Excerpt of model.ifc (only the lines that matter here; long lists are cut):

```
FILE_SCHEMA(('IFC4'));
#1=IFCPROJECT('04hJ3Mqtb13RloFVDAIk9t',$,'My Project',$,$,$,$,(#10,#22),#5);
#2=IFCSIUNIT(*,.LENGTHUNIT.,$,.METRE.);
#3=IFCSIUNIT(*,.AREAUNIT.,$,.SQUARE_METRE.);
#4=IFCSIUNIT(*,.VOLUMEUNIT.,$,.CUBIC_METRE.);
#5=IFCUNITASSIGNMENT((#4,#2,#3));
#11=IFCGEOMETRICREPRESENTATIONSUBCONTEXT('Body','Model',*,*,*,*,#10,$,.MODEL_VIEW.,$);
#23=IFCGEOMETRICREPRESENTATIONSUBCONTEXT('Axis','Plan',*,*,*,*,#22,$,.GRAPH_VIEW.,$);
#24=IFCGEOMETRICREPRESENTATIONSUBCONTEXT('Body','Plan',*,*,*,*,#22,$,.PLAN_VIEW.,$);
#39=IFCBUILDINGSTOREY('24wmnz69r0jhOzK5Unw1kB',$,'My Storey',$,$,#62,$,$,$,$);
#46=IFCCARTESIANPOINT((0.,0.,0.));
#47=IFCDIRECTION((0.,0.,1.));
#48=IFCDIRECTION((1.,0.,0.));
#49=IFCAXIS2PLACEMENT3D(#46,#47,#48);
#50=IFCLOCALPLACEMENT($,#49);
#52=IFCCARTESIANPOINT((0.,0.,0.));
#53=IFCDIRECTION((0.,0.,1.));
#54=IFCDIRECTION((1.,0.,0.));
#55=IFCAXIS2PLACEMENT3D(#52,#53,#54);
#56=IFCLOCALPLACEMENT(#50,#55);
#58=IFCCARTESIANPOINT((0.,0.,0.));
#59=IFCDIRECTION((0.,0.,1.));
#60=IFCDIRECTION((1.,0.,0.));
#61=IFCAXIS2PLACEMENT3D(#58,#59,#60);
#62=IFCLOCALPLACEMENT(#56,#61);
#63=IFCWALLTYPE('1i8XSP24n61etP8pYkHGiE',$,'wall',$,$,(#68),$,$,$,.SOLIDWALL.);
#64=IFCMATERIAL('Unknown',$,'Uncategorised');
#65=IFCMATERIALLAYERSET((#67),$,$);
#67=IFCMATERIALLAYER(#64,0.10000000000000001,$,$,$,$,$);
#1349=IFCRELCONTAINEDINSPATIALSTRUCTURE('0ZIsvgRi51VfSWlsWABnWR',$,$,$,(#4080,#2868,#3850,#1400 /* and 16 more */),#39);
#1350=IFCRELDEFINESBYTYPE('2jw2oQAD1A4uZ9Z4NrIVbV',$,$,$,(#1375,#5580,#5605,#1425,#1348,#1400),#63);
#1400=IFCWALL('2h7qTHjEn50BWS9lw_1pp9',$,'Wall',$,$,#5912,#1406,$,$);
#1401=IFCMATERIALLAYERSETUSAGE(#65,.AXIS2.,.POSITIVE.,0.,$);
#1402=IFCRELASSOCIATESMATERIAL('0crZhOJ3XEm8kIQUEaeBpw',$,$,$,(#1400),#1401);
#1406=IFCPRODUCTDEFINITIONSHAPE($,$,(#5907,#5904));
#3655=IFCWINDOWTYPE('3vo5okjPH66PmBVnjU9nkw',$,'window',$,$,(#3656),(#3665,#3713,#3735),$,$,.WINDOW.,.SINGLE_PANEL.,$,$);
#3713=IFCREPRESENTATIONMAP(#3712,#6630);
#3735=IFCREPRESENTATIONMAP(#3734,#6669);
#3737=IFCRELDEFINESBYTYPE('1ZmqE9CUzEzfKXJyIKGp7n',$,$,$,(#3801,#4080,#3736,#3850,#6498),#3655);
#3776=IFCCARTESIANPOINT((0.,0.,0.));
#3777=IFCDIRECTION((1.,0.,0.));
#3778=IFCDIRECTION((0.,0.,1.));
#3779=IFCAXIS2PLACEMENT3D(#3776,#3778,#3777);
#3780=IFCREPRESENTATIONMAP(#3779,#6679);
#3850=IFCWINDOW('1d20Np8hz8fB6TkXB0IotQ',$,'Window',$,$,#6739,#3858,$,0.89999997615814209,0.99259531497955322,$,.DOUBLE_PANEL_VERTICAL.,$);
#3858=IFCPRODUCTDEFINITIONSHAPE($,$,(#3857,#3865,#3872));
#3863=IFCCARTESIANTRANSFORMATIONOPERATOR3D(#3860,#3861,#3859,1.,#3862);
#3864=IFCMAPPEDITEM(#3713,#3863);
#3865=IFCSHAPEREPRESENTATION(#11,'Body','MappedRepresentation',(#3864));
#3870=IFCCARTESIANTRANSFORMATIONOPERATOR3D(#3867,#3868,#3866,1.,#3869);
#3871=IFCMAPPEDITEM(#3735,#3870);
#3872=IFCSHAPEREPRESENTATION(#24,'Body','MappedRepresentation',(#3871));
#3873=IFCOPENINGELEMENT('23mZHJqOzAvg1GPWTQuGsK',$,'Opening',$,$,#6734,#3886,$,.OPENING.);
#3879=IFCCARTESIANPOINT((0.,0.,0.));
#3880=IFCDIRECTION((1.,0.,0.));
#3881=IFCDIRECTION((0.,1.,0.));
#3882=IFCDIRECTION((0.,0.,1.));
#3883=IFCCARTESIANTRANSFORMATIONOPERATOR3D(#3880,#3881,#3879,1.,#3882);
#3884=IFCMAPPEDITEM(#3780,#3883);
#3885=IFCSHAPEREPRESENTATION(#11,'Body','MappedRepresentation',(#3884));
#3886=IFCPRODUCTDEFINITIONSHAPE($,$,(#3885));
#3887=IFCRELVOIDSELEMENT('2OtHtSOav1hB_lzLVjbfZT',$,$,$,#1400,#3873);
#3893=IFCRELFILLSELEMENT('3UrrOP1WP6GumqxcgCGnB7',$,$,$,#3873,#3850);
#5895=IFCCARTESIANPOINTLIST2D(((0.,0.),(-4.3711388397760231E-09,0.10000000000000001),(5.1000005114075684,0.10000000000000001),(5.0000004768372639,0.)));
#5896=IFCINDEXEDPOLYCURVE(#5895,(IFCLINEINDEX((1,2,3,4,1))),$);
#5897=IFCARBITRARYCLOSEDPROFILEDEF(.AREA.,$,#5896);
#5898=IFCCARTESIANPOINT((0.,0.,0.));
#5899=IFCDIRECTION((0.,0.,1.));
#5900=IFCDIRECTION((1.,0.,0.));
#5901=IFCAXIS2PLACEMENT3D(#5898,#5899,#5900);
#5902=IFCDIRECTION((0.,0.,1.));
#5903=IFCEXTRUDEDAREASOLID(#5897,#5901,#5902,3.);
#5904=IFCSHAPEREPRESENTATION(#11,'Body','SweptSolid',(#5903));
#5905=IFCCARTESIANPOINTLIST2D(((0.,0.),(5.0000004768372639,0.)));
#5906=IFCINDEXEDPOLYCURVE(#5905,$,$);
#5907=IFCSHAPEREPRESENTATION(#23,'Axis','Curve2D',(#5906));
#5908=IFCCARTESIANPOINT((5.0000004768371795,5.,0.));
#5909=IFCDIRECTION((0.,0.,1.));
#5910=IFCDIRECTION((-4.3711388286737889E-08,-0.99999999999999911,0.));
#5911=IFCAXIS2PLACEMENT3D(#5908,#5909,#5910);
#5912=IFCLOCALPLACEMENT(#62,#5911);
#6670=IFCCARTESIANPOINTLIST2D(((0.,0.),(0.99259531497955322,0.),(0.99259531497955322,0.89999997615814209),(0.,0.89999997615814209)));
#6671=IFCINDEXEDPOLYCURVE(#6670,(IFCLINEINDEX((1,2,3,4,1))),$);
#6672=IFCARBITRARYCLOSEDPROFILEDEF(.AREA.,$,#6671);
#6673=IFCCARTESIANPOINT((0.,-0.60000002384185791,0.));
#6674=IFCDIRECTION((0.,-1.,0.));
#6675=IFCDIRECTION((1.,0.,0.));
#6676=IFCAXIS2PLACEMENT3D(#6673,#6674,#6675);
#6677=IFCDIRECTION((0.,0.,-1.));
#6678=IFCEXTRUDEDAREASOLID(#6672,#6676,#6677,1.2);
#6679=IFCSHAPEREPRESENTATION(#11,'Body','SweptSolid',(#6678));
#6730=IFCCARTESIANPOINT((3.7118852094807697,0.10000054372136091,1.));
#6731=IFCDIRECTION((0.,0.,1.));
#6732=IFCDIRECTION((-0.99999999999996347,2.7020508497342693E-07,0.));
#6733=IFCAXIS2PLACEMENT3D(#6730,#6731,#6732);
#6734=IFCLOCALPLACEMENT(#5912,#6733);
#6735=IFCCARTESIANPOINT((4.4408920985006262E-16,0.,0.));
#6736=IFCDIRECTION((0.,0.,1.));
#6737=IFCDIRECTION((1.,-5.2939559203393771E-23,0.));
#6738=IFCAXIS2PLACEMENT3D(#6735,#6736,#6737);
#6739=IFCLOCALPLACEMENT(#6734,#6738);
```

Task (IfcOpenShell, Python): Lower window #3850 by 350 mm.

```python
import numpy as np
import ifcopenshell
import ifcopenshell.api.geometry
import ifcopenshell.util.placement
import ifcopenshell.util.unit

model = ifcopenshell.open("model.ifc")
unit_scale = ifcopenshell.util.unit.calculate_unit_scale(model)

window = model.by_guid("1d20Np8hz8fB6TkXB0IotQ")
opening = window.FillsVoids[0].RelatingOpeningElement
dz = -0.35 / unit_scale

shift = np.array([0.0, 0.0, dz])
# The window is placed relative to its opening, so it follows when the opening moves.
matrix = ifcopenshell.util.placement.get_local_placement(opening.ObjectPlacement)
matrix[:3, 3] += shift
ifcopenshell.api.geometry.edit_object_placement(
    model, product=opening, matrix=matrix, is_si=False, should_transform_children=True
)

print(f"moved by {dz * unit_scale:+.3f} m")

model.write("model_edited.ifc")
```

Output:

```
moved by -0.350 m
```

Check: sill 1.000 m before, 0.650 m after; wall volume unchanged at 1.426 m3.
